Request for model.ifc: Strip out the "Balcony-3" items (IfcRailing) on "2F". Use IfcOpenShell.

First a look at what the model holds.

```python
import ifcopenshell
import ifcopenshell.util.element

model = ifcopenshell.open("model.ifc")
print(model.schema)
storey = next(s for s in model.by_type("IfcBuildingStorey") if s.Name == "2F")
railings = [e for e in ifcopenshell.util.element.get_decomposition(storey) if e.is_a("IfcRailing")]
seen = {}
for e in railings:
    element_type = ifcopenshell.util.element.get_type(e)
    name = element_type.Name if element_type not in (None, e) else None
    seen[name] = seen.get(name, 0) + 1
for name, count in sorted(seen.items(), key=str):
    print(count, "x", name)
```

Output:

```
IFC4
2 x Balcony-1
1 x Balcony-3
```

```python
import ifcopenshell
import ifcopenshell.api.root
import ifcopenshell.util.element

model = ifcopenshell.open("model.ifc")

storey = next(s for s in model.by_type("IfcBuildingStorey") if s.Name == "2F")
railings = [e for e in ifcopenshell.util.element.get_decomposition(storey) if e.is_a("IfcRailing")]
targets = [e for e in railings if (t := ifcopenshell.util.element.get_type(e)) not in (None, e) and t.Name == "Balcony-3"]

for e in targets:
    ifcopenshell.api.root.remove_product(model, product=e)
print(len(targets), "removed")

model.write("model_updated.ifc")
```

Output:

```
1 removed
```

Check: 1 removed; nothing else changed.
